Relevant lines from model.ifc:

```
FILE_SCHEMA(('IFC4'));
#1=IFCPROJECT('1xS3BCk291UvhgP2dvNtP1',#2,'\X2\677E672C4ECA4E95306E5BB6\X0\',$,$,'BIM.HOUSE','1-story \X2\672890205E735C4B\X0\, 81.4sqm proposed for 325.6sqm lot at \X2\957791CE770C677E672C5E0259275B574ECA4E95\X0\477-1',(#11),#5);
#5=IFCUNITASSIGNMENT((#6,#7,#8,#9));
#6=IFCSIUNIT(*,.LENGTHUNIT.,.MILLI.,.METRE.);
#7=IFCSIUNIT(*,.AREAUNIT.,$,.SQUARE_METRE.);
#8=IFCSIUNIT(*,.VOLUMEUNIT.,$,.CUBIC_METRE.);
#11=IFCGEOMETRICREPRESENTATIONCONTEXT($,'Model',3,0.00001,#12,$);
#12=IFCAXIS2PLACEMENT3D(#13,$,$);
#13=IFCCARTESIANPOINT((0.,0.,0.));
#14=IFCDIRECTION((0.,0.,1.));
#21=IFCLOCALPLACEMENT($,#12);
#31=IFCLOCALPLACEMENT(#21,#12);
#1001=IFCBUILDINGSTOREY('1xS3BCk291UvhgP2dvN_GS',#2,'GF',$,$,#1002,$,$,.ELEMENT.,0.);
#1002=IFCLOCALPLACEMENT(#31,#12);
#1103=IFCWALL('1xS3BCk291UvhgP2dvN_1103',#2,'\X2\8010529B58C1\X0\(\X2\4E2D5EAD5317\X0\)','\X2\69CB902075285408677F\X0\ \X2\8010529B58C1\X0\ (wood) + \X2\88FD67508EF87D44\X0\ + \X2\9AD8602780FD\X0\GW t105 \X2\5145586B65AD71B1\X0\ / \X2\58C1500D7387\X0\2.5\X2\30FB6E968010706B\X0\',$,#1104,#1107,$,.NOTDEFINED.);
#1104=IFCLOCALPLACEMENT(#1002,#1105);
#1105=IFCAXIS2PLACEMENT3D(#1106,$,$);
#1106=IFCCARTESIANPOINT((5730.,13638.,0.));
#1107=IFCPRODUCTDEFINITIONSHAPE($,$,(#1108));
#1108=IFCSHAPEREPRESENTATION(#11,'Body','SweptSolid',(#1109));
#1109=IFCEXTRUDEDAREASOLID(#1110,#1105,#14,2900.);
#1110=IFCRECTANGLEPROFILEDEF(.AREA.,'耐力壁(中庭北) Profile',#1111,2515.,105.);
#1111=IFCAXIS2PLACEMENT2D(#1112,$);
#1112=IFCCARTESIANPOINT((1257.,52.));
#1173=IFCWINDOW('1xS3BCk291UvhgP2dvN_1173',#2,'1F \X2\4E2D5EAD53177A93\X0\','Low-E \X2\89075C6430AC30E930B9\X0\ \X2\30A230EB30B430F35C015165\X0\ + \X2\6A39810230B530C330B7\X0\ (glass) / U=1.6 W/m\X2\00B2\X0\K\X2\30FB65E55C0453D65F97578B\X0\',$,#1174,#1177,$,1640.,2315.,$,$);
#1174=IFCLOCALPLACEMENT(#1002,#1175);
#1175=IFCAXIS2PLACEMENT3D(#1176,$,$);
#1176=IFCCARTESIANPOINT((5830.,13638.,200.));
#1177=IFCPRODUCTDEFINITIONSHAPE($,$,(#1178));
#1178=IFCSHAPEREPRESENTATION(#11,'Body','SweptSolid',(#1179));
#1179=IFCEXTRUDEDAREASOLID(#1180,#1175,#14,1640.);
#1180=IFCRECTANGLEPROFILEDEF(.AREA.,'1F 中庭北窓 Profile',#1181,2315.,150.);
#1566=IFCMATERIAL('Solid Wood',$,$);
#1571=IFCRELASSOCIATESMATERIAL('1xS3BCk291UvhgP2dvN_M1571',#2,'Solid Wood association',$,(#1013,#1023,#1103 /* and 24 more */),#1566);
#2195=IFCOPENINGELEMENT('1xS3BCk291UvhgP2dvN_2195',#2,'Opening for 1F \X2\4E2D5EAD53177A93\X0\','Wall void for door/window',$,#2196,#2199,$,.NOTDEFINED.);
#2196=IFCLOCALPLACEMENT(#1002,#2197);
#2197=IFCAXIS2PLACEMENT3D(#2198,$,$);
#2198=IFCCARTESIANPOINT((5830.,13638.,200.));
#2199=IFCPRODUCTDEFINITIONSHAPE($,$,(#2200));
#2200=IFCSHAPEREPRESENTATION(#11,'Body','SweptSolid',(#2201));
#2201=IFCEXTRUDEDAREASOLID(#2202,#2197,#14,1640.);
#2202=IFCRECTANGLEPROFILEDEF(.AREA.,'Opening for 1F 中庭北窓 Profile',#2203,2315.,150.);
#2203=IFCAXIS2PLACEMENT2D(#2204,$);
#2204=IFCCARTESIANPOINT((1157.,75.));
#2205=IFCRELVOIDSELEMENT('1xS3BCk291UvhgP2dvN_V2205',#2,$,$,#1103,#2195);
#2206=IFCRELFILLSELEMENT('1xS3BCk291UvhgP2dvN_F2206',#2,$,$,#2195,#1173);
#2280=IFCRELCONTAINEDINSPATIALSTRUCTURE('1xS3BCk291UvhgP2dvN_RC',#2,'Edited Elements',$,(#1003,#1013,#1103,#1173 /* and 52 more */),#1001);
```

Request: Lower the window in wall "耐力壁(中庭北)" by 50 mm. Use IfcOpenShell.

```python
import numpy as np
import ifcopenshell
import ifcopenshell.api.geometry
import ifcopenshell.util.placement
import ifcopenshell.util.unit

model = ifcopenshell.open("model.ifc")
unit_scale = ifcopenshell.util.unit.calculate_unit_scale(model)

window = model.by_guid("1xS3BCk291UvhgP2dvN_1173")
opening = window.FillsVoids[0].RelatingOpeningElement
dz = -50.0

shift = np.array([0.0, 0.0, dz])
# The window is not placed relative to its opening, so move both.
for product in (opening, window):
    matrix = ifcopenshell.util.placement.get_local_placement(product.ObjectPlacement)
    matrix[:3, 3] += shift
    ifcopenshell.api.geometry.edit_object_placement(model, product=product, matrix=matrix, is_si=False)

print(f"moved by {dz * unit_scale:+.3f} m")

model.write("model_edited.ifc")
```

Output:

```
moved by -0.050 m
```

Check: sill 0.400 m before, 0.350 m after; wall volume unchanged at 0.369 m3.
